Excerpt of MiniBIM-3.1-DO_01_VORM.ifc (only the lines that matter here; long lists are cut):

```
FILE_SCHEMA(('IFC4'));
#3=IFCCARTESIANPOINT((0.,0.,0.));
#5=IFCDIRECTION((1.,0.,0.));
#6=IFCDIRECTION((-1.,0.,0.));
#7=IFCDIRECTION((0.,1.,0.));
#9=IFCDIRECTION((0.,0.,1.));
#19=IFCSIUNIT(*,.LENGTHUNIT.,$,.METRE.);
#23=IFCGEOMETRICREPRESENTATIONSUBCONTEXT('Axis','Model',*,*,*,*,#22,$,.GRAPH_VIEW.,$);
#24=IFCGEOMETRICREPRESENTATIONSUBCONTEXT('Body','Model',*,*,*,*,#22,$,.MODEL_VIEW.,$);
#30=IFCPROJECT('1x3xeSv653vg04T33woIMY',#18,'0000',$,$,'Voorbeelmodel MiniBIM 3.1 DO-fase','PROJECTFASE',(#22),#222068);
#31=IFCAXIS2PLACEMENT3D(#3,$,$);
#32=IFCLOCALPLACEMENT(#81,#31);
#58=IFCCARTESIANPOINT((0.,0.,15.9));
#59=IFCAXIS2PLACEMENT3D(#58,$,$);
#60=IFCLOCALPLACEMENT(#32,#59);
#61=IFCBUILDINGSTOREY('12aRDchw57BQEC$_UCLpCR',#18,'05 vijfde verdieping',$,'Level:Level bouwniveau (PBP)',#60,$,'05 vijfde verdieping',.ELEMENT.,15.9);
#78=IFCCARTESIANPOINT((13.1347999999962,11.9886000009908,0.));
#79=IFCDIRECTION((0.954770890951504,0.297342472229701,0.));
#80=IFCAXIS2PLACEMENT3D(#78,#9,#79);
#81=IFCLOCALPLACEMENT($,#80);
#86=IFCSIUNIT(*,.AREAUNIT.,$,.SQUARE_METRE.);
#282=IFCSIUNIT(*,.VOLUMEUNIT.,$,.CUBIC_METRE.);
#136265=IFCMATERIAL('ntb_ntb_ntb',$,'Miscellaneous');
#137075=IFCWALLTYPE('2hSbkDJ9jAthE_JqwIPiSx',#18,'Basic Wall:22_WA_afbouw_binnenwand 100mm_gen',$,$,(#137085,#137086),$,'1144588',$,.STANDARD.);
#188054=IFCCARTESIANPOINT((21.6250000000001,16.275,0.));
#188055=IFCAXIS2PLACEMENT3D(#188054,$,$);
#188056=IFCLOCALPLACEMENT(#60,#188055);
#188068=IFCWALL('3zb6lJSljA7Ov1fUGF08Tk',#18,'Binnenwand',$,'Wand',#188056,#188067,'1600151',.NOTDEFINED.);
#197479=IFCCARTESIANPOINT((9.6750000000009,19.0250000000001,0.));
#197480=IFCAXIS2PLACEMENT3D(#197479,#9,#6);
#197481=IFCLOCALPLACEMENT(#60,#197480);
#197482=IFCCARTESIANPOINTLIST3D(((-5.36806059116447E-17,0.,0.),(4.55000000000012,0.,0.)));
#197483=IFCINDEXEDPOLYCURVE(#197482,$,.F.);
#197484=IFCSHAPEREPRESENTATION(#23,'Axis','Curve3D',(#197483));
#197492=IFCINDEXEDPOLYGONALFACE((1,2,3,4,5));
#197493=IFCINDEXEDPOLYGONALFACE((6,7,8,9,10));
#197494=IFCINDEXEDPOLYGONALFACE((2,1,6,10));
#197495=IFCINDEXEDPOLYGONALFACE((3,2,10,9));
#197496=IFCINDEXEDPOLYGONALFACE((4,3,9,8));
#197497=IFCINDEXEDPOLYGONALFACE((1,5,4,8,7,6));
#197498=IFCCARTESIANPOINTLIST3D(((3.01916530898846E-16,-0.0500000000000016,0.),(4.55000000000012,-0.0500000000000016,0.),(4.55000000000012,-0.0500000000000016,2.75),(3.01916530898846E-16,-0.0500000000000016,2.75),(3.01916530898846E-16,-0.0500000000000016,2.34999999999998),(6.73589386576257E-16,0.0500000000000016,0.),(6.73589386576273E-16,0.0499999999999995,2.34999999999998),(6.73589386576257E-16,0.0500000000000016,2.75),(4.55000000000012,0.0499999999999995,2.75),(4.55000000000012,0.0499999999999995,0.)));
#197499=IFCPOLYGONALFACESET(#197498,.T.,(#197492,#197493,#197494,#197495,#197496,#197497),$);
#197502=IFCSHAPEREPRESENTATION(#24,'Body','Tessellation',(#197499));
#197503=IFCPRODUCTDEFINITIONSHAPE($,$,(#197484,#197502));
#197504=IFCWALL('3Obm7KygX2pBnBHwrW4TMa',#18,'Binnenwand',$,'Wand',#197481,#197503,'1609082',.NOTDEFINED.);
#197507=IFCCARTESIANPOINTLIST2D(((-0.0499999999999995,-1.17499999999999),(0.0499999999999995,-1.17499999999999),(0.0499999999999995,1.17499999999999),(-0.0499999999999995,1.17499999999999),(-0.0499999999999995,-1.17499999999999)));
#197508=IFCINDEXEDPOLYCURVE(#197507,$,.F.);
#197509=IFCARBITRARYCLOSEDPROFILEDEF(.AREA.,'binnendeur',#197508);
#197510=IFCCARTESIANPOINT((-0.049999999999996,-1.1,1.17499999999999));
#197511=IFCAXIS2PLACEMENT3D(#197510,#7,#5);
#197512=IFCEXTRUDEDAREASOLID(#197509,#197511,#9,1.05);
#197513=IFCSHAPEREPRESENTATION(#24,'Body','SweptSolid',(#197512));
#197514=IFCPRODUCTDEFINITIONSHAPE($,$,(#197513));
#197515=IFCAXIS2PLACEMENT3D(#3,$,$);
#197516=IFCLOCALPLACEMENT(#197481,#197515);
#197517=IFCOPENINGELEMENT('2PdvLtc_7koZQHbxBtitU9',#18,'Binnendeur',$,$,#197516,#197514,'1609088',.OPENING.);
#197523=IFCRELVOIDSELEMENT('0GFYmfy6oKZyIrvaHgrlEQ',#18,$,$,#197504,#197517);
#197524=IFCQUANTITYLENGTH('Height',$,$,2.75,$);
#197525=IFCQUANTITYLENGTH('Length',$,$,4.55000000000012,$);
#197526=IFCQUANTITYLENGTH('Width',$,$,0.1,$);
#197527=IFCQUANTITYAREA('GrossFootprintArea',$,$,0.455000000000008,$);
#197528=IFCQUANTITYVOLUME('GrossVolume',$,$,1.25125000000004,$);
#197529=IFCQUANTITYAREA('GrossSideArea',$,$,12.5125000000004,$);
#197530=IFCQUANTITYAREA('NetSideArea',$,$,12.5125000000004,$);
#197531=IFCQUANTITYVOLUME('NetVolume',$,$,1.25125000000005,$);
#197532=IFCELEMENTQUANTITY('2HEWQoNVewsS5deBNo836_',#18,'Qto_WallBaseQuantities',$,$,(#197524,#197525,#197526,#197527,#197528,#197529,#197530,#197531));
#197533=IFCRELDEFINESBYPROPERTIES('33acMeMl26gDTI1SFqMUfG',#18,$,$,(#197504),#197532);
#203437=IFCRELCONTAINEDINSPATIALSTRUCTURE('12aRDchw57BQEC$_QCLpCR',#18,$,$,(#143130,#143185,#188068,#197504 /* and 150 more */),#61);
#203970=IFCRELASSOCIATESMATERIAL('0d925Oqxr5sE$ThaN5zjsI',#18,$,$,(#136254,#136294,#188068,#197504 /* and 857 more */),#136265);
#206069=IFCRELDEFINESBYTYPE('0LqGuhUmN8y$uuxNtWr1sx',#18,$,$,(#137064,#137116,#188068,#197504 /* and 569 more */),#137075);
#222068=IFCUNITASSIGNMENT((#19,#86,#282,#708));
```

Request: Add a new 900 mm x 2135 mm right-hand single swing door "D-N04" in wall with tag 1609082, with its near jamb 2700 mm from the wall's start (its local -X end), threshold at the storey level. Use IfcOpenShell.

```python
import numpy as np
import ifcopenshell
import ifcopenshell.api.feature
import ifcopenshell.api.geometry
import ifcopenshell.api.pset
import ifcopenshell.api.root
import ifcopenshell.api.spatial
import ifcopenshell.geom
import ifcopenshell.util.element
import ifcopenshell.util.placement
import ifcopenshell.util.representation
import ifcopenshell.util.shape
import ifcopenshell.util.unit

model = ifcopenshell.open("MiniBIM-3.1-DO_01_VORM.ifc")
unit_scale = ifcopenshell.util.unit.calculate_unit_scale(model)
area_scale = ifcopenshell.util.unit.calculate_unit_scale(model, "AREAUNIT")
volume_scale = ifcopenshell.util.unit.calculate_unit_scale(model, "VOLUMEUNIT")
settings = ifcopenshell.geom.settings()


def volume(element):
    """Net volume in cubic metres, openings subtracted."""
    shape = ifcopenshell.geom.create_shape(settings, element)
    return ifcopenshell.util.shape.get_volume(shape.geometry)


wall = model.by_id(197504)
storey = ifcopenshell.util.element.get_container(wall, ifc_class="IfcBuildingStorey")
context = ifcopenshell.util.representation.get_context(model, "Model", "Body", "MODEL_VIEW")
before = volume(wall)

width, height, from_end, sill = 0.9, 2.135, 2.7, 0.0  # metres

# The wall runs along its own X axis, and the end named is its -X end.
wall_shape = ifcopenshell.geom.create_shape(settings, wall)
x, y, z = ifcopenshell.util.shape.get_vertices(wall_shape.geometry).T
start = x.min() + from_end
face, thickness = float(y.min()), float(y.max() - y.min())
wall_matrix = ifcopenshell.util.placement.get_local_placement(wall.ObjectPlacement)
level = ifcopenshell.util.placement.get_local_placement(storey.ObjectPlacement)[2, 3]


def in_wall(x, y):
    """Placement at x, y metres in the wall's axes, at sill height."""
    matrix = wall_matrix.copy()
    matrix[:, 3] = wall_matrix @ np.array([x / unit_scale, y / unit_scale, 0.0, 1.0])
    matrix[2, 3] = level + sill / unit_scale
    return matrix


# Opening: a box that overshoots both wall faces by 50 mm.
opening = ifcopenshell.api.root.create_entity(model, ifc_class="IfcOpeningElement", predefined_type="OPENING")
box = ifcopenshell.api.geometry.add_wall_representation(
    model, context=context, length=width, height=height, thickness=thickness + 0.1
)
ifcopenshell.api.geometry.assign_representation(model, product=opening, representation=box)
ifcopenshell.api.geometry.edit_object_placement(model, product=opening, matrix=in_wall(start, face - 0.05), is_si=False)
ifcopenshell.api.feature.add_feature(model, feature=opening, element=wall)

door = ifcopenshell.api.root.create_entity(model, ifc_class="IfcDoor", name="D-N04", predefined_type="DOOR")
door.OverallWidth, door.OverallHeight = width / unit_scale, height / unit_scale
door.OperationType = "SINGLE_SWING_RIGHT"
body = ifcopenshell.api.geometry.add_door_representation(
    model,
    context=context,
    overall_width=door.OverallWidth,
    overall_height=door.OverallHeight,
    operation_type="SINGLE_SWING_RIGHT",
    lining_properties={"LiningDepth": thickness / unit_scale, "ThresholdDepth": thickness / unit_scale},
)
ifcopenshell.api.geometry.assign_representation(model, product=door, representation=body)
ifcopenshell.api.spatial.assign_container(model, products=[door], relating_structure=storey)
ifcopenshell.api.feature.add_filling(model, opening=opening, element=door)

# The lining spans the wall, so the door starts at the wall face.
ifcopenshell.api.geometry.edit_object_placement(model, product=door, matrix=in_wall(start, face), is_si=False)

after = volume(wall)

# Update the wall's stored quantities.
qto = model.by_id(ifcopenshell.util.element.get_pset(wall, "Qto_WallBaseQuantities", should_inherit=False)["id"])
ifcopenshell.api.pset.edit_qto(model, qto=qto, properties={
    "NetSideArea": after / thickness / area_scale,
    "NetVolume": after / volume_scale,
})

print(f"wall volume {before:.3f} -> {after:.3f} m3")

model.write("MiniBIM-3.1-DO_01_VORM-out.ifc")
```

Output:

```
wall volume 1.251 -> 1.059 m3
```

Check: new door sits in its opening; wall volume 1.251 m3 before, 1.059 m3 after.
